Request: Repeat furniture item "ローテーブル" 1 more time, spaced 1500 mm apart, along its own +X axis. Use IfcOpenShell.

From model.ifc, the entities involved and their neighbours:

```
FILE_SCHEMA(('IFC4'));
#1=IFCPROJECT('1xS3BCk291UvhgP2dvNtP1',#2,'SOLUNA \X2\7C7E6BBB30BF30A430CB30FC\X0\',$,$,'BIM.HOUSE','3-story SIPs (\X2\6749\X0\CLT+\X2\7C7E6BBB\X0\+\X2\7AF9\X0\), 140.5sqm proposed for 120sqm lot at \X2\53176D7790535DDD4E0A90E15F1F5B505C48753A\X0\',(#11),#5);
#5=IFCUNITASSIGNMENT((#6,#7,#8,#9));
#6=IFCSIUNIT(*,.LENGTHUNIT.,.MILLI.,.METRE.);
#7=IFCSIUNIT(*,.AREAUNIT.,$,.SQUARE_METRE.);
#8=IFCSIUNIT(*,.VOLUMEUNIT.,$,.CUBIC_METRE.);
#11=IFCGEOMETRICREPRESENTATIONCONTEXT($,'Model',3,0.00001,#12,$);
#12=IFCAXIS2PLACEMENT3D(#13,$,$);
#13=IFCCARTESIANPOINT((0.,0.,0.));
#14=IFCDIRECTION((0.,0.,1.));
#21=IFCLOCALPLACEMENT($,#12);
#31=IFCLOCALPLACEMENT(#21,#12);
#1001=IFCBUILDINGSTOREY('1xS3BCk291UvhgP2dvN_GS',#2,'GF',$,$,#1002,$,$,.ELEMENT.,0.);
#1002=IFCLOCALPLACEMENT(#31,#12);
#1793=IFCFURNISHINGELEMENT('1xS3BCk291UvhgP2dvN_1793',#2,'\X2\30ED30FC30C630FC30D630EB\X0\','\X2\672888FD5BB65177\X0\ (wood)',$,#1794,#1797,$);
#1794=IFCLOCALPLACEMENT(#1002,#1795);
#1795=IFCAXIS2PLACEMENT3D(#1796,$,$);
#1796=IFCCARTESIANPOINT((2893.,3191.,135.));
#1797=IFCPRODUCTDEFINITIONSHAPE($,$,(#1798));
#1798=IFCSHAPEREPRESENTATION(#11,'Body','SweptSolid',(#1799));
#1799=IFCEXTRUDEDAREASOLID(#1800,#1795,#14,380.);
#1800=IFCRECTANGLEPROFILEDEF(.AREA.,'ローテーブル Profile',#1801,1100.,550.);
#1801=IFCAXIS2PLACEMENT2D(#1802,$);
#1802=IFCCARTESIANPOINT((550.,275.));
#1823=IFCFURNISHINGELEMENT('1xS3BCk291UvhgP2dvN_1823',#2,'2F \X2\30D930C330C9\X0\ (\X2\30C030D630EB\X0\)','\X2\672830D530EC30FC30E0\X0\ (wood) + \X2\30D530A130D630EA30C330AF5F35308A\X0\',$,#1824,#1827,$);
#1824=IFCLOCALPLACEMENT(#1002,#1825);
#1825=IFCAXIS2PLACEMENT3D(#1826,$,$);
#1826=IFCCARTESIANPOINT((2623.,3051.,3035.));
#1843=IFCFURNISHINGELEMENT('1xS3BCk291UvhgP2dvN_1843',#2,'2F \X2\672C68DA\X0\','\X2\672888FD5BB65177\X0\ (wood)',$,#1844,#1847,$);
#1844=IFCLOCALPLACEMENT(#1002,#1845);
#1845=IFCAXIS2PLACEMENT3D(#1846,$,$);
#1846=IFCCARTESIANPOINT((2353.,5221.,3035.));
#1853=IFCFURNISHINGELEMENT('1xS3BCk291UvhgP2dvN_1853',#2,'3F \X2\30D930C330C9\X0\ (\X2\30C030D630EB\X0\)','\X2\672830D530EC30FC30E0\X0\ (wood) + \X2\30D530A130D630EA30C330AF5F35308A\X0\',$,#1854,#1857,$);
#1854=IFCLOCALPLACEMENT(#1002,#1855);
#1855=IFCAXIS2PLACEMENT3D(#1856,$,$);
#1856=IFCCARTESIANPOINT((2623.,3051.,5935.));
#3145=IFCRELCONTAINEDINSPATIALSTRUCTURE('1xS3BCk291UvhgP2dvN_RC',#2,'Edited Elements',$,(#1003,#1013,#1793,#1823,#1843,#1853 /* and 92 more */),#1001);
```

```python
import ifcopenshell
import ifcopenshell.api.geometry
import ifcopenshell.api.root
import ifcopenshell.util.element
import ifcopenshell.util.placement
import ifcopenshell.util.unit

model = ifcopenshell.open("model.ifc")
unit_scale = ifcopenshell.util.unit.calculate_unit_scale(model)


def reuse_history(source, copy):
    """copy_class also copies each property set's owner history, people and application; keep the originals."""
    for rel in copy.IsDefinedBy:
        if rel.is_a("IfcRelDefinesByProperties") and (history := rel.RelatingPropertyDefinition.OwnerHistory):
            rel.RelatingPropertyDefinition.OwnerHistory = source.OwnerHistory
            ifcopenshell.util.element.remove_deep2(model, history)


source = model.by_id(1793)
base = ifcopenshell.util.placement.get_local_placement(source.ObjectPlacement)
step = base[:3, 0] * 1.5 / unit_scale

for i in range(1, 2):
    copy = ifcopenshell.api.root.copy_class(model, product=source)
    copy.Representation = ifcopenshell.util.element.copy_deep(
        model, source.Representation, exclude=["IfcGeometricRepresentationContext", "IfcRepresentationMap"]
    )
    reuse_history(source, copy)
    matrix = base.copy()
    matrix[:3, 3] += i * step
    print("added at", matrix[:3, 3].round(3) + 0.0)
    ifcopenshell.api.geometry.edit_object_placement(model, product=copy, matrix=matrix, is_si=False)

model.write("model_edited.ifc")
```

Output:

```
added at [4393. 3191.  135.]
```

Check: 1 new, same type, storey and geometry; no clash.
